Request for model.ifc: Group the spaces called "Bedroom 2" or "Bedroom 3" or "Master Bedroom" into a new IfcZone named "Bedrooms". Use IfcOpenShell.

First a look at what the model holds.

```python
import ifcopenshell

model = ifcopenshell.open("model.ifc")
print(model.schema)
seen = {}
for space in model.by_type("IfcSpace"):
    seen[space.LongName] = seen.get(space.LongName, 0) + 1
for name, count in sorted(seen.items(), key=str):
    print(count, "x", name)
print("zones:", [z.Name for z in model.by_type("IfcZone")][:20])
```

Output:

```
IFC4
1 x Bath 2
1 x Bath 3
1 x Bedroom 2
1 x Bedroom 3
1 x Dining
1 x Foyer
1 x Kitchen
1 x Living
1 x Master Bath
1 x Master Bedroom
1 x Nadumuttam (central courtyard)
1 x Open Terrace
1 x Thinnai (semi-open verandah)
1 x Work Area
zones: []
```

```python
import ifcopenshell
import ifcopenshell.api.group
import ifcopenshell.api.root

model = ifcopenshell.open("model.ifc")

names = {"Bedroom 2", "Bedroom 3", "Master Bedroom"}
spaces = [s for s in model.by_type("IfcSpace") if s.LongName in names]

zone = ifcopenshell.api.root.create_entity(model, ifc_class="IfcZone", name="Bedrooms")
ifcopenshell.api.group.assign_group(model, products=spaces, group=zone)
print(len(spaces), "spaces in", zone.Name)

model.write("model_rev.ifc")
```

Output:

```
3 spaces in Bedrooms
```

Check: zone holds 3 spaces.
